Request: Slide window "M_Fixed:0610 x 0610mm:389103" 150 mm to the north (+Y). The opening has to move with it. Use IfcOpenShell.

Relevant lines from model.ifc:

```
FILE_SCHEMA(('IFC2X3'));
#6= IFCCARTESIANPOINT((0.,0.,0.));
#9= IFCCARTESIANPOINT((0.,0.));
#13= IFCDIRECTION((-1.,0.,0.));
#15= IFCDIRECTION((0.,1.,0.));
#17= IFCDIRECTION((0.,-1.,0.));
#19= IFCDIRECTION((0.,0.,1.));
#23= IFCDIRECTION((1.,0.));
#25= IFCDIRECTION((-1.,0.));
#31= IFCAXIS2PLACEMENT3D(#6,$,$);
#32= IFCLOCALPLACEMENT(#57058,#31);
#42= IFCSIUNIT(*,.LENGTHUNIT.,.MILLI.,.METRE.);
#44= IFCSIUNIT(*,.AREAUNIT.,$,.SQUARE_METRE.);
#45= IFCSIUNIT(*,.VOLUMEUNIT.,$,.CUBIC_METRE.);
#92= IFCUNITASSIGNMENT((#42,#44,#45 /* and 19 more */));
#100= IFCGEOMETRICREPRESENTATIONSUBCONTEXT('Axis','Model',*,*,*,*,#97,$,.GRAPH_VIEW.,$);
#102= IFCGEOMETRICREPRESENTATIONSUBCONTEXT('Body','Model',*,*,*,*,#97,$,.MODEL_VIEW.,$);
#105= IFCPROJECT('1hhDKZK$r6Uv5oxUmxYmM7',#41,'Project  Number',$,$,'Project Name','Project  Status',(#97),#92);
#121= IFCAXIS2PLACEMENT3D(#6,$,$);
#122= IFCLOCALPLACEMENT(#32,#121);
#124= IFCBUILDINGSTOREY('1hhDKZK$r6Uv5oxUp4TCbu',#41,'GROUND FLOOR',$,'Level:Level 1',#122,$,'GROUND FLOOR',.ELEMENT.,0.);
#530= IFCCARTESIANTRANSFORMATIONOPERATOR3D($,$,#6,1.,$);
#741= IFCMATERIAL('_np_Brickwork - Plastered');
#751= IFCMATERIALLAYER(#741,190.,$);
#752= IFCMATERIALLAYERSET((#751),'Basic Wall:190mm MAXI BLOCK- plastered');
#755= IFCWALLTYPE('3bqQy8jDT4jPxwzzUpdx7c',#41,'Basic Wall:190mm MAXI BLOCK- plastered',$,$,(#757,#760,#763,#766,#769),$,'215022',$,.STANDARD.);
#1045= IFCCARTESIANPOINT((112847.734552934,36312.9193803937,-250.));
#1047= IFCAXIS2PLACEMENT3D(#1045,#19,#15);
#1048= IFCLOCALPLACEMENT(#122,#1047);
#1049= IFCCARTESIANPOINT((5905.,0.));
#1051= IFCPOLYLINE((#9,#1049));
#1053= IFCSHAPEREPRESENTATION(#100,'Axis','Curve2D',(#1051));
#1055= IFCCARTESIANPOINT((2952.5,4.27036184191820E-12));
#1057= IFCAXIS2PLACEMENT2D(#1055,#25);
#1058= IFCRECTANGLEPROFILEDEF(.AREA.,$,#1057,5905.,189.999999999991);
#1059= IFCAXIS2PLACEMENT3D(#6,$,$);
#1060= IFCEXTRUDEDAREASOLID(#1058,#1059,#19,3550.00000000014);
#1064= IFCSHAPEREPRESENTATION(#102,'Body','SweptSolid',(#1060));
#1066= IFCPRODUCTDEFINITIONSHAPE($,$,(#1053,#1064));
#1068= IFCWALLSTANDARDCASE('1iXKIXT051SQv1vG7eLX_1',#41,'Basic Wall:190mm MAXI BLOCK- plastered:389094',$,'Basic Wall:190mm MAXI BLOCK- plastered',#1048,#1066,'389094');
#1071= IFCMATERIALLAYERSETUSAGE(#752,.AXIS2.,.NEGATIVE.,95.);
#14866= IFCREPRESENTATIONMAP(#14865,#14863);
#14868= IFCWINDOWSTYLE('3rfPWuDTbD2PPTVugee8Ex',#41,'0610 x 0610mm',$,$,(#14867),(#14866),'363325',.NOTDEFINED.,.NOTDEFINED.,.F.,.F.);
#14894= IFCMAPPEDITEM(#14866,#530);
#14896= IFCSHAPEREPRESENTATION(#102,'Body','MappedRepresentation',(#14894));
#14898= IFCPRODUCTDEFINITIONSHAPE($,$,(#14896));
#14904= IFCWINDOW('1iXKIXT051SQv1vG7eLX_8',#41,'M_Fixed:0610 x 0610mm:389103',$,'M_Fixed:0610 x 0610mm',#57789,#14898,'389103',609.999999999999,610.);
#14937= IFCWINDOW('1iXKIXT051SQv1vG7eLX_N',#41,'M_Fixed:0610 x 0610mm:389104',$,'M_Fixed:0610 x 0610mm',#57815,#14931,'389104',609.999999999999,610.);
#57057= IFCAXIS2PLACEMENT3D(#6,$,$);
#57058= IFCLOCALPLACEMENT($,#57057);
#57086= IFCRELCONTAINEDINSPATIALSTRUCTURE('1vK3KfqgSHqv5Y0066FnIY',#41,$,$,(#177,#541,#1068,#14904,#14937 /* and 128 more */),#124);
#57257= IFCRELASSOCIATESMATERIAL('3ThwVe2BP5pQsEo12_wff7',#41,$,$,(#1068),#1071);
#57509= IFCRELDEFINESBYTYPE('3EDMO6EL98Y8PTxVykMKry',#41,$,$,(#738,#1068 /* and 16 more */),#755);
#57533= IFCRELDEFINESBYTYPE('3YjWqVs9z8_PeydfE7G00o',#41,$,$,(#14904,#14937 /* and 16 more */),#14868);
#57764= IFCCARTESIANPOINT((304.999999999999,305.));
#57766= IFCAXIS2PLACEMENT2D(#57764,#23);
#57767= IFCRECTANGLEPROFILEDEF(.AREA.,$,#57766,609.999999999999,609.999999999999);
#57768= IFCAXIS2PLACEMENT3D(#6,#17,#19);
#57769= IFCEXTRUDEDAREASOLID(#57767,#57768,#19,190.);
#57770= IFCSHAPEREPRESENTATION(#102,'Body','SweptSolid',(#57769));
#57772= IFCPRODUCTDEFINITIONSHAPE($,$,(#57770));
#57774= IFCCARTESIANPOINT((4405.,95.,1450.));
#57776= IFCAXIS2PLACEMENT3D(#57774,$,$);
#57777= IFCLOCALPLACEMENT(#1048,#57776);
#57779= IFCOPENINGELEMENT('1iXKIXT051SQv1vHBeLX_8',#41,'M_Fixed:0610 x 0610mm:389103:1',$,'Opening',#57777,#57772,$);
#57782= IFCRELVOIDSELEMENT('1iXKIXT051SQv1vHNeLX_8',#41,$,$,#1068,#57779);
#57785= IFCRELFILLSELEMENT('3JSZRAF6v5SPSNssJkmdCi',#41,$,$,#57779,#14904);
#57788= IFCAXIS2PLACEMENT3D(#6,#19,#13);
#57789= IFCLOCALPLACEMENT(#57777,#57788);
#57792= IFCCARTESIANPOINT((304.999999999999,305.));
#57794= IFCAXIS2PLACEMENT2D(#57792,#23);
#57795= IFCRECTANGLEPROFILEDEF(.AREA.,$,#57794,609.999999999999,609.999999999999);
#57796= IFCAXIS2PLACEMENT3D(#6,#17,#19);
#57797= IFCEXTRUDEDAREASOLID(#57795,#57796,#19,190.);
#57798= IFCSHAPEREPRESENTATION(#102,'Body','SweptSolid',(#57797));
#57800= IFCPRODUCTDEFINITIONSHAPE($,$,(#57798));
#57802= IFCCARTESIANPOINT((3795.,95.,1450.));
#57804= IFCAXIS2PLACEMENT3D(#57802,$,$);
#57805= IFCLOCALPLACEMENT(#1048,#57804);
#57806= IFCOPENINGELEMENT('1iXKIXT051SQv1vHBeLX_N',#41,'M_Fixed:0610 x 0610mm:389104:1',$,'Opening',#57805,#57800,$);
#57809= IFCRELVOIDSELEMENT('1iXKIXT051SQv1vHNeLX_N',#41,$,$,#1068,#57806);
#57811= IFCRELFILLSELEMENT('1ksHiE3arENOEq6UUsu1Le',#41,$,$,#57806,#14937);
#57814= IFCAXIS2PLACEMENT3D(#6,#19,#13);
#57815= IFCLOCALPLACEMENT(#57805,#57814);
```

```python
import ifcopenshell
import ifcopenshell.api.geometry
import ifcopenshell.util.placement

model = ifcopenshell.open("model.ifc")

window = model.by_guid("1iXKIXT051SQv1vG7eLX_8")
opening = window.FillsVoids[0].RelatingOpeningElement
wall = opening.VoidsElements[0].RelatingBuildingElement

wall_matrix = ifcopenshell.util.placement.get_local_placement(wall.ObjectPlacement)
shift = wall_matrix[:3, 0] * 150.0
before = ifcopenshell.util.placement.get_local_placement(window.ObjectPlacement)[:3, 3].copy()

# The window is placed relative to its opening, so it follows when the opening moves.
matrix = ifcopenshell.util.placement.get_local_placement(opening.ObjectPlacement)
matrix[:3, 3] += shift
ifcopenshell.api.geometry.edit_object_placement(
    model, product=opening, matrix=matrix, is_si=False, should_transform_children=True
)

after = ifcopenshell.util.placement.get_local_placement(window.ObjectPlacement)[:3, 3]
print("window moved by", (after - before).round(3) + 0.0)

model.write("model-out.ifc")
```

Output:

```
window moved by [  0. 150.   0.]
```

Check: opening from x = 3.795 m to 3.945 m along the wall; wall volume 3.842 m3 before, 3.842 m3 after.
